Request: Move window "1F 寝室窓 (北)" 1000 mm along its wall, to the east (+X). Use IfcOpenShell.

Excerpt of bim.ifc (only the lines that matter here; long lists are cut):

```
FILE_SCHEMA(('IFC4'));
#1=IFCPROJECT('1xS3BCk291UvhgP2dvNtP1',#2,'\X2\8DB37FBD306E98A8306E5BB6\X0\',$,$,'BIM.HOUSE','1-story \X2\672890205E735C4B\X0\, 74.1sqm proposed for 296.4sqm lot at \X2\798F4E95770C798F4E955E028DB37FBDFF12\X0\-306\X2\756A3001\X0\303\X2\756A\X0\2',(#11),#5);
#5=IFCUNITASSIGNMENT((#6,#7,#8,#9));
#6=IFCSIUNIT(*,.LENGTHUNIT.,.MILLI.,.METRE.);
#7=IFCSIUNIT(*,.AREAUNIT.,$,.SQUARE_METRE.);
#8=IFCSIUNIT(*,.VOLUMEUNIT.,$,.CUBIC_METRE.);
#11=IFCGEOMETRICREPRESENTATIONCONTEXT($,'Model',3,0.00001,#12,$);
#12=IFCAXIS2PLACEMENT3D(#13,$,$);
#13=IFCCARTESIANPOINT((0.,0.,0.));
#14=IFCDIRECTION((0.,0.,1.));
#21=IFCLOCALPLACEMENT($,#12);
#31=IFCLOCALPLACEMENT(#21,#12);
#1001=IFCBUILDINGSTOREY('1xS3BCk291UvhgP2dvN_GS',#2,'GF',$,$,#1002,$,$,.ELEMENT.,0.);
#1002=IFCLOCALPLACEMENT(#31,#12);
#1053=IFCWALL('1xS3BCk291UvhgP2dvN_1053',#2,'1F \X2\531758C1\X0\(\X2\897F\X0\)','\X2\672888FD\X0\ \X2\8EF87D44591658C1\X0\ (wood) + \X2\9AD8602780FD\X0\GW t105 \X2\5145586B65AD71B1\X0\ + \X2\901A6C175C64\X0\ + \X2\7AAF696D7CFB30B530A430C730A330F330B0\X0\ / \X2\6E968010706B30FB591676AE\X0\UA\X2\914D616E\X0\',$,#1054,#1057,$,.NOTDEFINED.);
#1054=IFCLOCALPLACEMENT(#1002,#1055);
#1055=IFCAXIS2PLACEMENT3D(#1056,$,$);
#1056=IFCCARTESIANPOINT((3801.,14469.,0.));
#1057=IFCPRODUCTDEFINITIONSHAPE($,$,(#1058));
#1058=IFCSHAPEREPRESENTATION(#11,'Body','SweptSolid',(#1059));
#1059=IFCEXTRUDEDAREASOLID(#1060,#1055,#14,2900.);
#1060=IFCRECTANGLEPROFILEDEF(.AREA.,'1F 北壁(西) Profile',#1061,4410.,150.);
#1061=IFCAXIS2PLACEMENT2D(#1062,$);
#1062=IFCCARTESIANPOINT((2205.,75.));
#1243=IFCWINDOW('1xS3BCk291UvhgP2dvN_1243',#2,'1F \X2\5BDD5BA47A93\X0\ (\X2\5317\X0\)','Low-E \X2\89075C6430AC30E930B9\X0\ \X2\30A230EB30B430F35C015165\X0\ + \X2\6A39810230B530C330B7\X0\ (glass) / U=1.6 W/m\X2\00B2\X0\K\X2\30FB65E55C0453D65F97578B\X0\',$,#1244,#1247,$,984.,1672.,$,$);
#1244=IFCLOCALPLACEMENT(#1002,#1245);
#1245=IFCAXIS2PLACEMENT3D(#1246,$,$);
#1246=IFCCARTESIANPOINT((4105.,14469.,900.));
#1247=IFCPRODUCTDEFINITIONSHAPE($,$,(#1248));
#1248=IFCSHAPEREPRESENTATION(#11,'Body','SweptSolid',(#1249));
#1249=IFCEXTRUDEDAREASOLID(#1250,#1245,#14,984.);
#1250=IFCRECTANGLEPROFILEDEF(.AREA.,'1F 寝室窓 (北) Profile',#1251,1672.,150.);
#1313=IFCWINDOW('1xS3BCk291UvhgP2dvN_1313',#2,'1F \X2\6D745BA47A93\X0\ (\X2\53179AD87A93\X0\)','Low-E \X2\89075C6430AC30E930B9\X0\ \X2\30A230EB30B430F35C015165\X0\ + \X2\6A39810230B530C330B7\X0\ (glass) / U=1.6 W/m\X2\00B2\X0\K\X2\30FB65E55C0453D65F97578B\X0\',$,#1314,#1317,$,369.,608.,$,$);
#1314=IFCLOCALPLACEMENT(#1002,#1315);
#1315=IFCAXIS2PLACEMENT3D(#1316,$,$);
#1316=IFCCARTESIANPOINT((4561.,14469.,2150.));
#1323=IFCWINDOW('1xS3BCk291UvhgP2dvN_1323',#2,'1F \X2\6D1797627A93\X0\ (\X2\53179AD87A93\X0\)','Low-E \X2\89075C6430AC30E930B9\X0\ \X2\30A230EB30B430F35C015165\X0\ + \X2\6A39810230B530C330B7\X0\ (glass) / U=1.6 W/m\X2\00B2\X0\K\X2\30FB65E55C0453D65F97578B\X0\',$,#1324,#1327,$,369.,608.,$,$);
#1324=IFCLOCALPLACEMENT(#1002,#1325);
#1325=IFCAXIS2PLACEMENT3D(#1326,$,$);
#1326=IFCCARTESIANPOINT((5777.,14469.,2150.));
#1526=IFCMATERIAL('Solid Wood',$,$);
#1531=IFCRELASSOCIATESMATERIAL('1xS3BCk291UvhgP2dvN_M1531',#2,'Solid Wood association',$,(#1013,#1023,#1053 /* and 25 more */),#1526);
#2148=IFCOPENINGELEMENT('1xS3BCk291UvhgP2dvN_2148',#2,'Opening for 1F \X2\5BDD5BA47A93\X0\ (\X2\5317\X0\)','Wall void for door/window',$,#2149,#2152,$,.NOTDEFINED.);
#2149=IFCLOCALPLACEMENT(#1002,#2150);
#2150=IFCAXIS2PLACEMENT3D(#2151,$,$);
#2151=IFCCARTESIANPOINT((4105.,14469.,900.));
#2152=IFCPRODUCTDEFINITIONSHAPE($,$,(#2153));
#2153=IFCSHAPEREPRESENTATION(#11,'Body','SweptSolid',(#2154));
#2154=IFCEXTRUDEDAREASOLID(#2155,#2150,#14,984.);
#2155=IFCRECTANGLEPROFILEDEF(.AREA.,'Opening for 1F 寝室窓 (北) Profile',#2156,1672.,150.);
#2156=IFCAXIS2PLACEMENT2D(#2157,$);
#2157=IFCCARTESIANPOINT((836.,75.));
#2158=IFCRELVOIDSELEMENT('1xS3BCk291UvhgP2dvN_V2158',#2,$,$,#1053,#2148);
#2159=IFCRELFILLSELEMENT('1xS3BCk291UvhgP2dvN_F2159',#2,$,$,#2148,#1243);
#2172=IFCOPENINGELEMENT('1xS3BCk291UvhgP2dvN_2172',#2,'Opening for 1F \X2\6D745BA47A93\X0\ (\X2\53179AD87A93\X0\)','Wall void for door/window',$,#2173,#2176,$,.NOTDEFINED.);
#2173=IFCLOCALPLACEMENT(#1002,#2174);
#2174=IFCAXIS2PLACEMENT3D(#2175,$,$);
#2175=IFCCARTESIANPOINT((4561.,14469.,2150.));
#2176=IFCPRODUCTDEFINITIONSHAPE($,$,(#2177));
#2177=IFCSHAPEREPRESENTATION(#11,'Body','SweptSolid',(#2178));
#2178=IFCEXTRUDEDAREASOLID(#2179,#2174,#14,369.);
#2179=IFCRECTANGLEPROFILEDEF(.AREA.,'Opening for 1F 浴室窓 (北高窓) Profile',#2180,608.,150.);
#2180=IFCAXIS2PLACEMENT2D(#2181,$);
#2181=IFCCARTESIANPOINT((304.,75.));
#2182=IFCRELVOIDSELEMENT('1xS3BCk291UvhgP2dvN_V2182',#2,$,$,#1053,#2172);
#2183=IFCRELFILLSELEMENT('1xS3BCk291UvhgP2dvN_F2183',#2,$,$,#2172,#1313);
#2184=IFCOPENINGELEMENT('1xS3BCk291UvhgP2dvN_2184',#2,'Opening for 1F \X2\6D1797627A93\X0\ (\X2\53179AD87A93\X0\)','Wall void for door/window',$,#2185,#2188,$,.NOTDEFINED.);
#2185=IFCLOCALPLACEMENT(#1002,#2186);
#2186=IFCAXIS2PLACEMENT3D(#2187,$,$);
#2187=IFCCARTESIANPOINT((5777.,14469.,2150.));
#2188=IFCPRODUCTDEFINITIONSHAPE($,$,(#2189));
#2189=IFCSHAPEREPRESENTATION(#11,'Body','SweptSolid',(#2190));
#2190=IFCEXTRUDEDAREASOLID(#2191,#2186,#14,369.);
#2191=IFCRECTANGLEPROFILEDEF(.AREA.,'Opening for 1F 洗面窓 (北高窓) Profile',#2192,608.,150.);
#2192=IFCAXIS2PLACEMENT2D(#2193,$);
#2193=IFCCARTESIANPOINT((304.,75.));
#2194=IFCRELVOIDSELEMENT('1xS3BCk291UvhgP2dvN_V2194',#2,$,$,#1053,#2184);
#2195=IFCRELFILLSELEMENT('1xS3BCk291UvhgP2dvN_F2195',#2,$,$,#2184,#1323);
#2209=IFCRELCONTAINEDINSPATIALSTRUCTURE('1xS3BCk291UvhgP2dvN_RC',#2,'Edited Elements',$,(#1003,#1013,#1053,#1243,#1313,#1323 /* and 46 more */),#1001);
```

```python
import ifcopenshell
import ifcopenshell.api.geometry
import ifcopenshell.util.placement
import ifcopenshell.util.unit

model = ifcopenshell.open("bim.ifc")
unit_scale = ifcopenshell.util.unit.calculate_unit_scale(model)

window = model.by_guid("1xS3BCk291UvhgP2dvN_1243")
opening = window.FillsVoids[0].RelatingOpeningElement
wall = opening.VoidsElements[0].RelatingBuildingElement

wall_matrix = ifcopenshell.util.placement.get_local_placement(wall.ObjectPlacement)
shift = wall_matrix[:3, 0] * 1 / unit_scale
before = ifcopenshell.util.placement.get_local_placement(window.ObjectPlacement)[:3, 3].copy()

# The window is not placed relative to its opening, so move both.
for product in (opening, window):
    matrix = ifcopenshell.util.placement.get_local_placement(product.ObjectPlacement)
    matrix[:3, 3] += shift
    ifcopenshell.api.geometry.edit_object_placement(model, product=product, matrix=matrix, is_si=False)

after = ifcopenshell.util.placement.get_local_placement(window.ObjectPlacement)[:3, 3]
print("window moved by", (after - before).round(3) + 0.0)

model.write("bim_rev.ifc")
```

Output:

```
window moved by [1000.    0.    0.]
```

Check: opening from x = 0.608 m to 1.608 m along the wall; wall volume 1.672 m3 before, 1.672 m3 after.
